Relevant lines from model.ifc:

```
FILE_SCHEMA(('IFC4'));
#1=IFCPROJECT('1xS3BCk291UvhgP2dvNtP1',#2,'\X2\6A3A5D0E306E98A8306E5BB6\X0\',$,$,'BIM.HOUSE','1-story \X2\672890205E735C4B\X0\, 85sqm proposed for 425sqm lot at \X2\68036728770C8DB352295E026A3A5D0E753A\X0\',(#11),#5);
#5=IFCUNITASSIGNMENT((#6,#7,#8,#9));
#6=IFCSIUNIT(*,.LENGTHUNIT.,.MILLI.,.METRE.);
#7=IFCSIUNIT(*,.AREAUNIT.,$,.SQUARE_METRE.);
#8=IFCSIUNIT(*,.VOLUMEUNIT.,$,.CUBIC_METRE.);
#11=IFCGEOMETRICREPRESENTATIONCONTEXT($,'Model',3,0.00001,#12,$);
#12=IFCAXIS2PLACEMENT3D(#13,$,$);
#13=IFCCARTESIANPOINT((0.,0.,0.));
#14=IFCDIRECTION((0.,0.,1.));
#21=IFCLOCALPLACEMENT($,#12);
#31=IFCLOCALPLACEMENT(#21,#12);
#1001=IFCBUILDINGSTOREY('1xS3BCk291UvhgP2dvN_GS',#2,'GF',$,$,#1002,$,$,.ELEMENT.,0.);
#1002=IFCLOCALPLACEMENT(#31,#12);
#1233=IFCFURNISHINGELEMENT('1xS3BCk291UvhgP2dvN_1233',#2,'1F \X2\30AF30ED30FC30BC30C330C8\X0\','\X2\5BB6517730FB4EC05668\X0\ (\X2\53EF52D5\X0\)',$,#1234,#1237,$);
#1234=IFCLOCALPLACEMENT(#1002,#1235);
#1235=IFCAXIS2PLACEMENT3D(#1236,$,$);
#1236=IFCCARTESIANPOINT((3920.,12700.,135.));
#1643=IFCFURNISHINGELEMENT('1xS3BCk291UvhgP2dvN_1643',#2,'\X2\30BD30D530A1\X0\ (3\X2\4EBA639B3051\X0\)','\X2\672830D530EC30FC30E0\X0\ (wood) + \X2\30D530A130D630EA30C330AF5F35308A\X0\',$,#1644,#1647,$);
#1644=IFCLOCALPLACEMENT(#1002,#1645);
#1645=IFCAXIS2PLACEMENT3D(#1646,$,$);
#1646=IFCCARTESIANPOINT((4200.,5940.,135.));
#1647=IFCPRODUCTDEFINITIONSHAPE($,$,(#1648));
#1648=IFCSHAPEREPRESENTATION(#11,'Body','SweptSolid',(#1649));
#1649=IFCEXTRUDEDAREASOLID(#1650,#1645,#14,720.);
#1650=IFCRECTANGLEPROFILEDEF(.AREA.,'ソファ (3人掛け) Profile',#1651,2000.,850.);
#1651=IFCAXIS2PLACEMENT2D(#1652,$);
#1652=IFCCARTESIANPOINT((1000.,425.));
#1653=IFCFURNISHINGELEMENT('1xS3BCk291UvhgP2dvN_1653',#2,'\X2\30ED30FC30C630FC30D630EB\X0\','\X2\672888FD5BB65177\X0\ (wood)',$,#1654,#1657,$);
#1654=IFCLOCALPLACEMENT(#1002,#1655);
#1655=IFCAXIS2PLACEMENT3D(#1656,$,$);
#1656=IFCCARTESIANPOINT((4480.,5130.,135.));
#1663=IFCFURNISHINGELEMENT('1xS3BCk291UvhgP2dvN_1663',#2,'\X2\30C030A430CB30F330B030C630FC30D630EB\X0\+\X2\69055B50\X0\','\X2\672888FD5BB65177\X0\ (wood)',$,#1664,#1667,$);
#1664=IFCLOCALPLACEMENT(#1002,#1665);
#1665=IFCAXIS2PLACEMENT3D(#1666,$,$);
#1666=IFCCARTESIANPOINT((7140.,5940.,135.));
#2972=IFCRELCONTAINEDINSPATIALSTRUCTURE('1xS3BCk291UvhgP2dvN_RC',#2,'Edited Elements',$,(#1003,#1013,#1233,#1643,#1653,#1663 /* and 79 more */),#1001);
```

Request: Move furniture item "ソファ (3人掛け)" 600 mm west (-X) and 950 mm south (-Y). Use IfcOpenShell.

```python
import ifcopenshell
import ifcopenshell.api.geometry
import ifcopenshell.util.placement
import ifcopenshell.util.unit

model = ifcopenshell.open("model.ifc")
unit_scale = ifcopenshell.util.unit.calculate_unit_scale(model)

item = model.by_id(1643)
matrix = ifcopenshell.util.placement.get_local_placement(item.ObjectPlacement)
matrix[0, 3] -= 0.6 / unit_scale
matrix[1, 3] -= 0.95 / unit_scale
ifcopenshell.api.geometry.edit_object_placement(model, product=item, matrix=matrix, is_si=False)

print(ifcopenshell.util.placement.get_local_placement(item.ObjectPlacement).round(3) + 0.0)

model.write("model_rev.ifc")
```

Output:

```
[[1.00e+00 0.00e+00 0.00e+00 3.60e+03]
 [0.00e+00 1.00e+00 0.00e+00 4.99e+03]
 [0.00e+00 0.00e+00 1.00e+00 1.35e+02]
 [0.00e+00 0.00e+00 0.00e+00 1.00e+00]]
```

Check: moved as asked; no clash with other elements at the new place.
